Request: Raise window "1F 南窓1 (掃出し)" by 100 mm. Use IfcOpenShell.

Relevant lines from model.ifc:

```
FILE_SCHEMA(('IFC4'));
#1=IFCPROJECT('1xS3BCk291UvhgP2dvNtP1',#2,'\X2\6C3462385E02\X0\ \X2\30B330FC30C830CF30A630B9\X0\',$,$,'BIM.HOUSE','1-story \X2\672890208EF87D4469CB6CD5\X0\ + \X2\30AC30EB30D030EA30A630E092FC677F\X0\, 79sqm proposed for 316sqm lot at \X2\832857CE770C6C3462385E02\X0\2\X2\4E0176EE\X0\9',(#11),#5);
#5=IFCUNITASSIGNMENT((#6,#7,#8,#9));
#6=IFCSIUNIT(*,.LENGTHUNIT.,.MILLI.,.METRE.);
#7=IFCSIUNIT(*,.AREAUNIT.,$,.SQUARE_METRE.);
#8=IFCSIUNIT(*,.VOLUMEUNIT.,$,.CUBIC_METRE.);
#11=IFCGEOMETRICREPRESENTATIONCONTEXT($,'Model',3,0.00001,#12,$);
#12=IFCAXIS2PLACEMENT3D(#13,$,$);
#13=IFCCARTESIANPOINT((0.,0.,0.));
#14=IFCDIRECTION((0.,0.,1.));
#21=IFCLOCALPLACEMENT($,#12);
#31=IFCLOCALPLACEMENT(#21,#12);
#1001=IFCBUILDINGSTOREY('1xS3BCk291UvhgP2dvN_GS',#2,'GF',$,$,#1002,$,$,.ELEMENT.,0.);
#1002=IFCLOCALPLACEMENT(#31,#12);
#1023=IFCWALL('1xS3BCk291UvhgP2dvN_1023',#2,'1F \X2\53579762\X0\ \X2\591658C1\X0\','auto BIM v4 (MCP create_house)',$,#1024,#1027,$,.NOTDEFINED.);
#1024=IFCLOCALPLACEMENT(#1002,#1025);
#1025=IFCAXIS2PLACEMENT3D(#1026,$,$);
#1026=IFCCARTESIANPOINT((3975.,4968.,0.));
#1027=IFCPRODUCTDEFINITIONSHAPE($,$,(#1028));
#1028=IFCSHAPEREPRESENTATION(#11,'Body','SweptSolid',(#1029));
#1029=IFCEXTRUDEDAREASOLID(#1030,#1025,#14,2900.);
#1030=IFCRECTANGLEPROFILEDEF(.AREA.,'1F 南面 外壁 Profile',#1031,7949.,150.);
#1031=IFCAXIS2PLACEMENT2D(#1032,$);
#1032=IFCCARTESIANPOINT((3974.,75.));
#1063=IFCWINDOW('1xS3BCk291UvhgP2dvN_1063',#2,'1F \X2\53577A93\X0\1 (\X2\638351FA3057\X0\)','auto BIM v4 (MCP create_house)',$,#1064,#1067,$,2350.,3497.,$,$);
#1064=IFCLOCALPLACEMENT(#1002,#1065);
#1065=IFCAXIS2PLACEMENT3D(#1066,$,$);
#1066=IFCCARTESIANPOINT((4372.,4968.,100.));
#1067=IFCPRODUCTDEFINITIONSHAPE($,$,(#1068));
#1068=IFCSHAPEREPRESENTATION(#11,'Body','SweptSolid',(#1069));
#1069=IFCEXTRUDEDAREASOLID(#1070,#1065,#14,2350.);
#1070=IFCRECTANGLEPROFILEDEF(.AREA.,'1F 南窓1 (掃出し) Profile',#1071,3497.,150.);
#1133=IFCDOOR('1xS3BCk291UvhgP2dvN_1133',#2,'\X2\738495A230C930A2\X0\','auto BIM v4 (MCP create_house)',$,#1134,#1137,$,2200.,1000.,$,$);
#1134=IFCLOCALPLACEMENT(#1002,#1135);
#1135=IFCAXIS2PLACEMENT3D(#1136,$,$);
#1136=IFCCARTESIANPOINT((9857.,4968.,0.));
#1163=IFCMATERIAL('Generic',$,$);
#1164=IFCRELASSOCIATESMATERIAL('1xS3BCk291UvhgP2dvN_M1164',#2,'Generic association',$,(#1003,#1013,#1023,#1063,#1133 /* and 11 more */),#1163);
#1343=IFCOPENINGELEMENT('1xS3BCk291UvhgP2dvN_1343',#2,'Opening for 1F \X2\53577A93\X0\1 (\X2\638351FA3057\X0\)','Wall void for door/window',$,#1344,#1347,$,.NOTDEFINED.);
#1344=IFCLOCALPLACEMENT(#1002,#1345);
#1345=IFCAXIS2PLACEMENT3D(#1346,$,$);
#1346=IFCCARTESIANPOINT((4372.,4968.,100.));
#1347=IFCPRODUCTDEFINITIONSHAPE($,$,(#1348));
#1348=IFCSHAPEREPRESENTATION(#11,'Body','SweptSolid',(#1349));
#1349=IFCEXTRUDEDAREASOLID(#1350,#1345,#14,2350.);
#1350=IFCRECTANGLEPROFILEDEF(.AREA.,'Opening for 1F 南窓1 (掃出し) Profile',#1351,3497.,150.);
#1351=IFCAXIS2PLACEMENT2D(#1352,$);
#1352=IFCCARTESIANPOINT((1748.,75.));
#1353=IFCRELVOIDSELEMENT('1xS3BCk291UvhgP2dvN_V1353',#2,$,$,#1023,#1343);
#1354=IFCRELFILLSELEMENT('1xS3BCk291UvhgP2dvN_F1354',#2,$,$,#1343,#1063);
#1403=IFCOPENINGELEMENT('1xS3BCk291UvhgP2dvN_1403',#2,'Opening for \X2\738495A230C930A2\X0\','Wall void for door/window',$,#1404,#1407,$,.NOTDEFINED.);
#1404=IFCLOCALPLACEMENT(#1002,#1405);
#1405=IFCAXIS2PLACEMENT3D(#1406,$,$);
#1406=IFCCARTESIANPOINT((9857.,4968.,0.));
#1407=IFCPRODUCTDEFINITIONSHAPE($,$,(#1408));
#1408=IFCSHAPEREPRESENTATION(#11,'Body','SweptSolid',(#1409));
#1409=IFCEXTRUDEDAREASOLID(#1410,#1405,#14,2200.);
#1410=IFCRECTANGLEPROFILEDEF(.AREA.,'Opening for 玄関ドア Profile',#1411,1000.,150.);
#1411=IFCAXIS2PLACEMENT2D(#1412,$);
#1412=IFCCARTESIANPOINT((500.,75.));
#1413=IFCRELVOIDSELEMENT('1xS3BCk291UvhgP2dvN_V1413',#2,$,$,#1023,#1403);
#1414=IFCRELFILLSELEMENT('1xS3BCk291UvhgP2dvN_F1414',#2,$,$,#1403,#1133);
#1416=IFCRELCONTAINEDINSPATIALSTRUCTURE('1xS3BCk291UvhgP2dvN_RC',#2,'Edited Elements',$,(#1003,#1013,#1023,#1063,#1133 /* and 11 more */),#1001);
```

```python
import numpy as np
import ifcopenshell
import ifcopenshell.api.geometry
import ifcopenshell.util.placement
import ifcopenshell.util.unit

model = ifcopenshell.open("model.ifc")
unit_scale = ifcopenshell.util.unit.calculate_unit_scale(model)

window = model.by_guid("1xS3BCk291UvhgP2dvN_1063")
opening = window.FillsVoids[0].RelatingOpeningElement
dz = 100.0

shift = np.array([0.0, 0.0, dz])
# The window is not placed relative to its opening, so move both.
for product in (opening, window):
    matrix = ifcopenshell.util.placement.get_local_placement(product.ObjectPlacement)
    matrix[:3, 3] += shift
    ifcopenshell.api.geometry.edit_object_placement(model, product=product, matrix=matrix, is_si=False)

print(f"moved by {dz * unit_scale:+.3f} m")

model.write("model_updated.ifc")
```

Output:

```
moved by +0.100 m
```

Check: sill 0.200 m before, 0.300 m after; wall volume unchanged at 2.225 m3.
